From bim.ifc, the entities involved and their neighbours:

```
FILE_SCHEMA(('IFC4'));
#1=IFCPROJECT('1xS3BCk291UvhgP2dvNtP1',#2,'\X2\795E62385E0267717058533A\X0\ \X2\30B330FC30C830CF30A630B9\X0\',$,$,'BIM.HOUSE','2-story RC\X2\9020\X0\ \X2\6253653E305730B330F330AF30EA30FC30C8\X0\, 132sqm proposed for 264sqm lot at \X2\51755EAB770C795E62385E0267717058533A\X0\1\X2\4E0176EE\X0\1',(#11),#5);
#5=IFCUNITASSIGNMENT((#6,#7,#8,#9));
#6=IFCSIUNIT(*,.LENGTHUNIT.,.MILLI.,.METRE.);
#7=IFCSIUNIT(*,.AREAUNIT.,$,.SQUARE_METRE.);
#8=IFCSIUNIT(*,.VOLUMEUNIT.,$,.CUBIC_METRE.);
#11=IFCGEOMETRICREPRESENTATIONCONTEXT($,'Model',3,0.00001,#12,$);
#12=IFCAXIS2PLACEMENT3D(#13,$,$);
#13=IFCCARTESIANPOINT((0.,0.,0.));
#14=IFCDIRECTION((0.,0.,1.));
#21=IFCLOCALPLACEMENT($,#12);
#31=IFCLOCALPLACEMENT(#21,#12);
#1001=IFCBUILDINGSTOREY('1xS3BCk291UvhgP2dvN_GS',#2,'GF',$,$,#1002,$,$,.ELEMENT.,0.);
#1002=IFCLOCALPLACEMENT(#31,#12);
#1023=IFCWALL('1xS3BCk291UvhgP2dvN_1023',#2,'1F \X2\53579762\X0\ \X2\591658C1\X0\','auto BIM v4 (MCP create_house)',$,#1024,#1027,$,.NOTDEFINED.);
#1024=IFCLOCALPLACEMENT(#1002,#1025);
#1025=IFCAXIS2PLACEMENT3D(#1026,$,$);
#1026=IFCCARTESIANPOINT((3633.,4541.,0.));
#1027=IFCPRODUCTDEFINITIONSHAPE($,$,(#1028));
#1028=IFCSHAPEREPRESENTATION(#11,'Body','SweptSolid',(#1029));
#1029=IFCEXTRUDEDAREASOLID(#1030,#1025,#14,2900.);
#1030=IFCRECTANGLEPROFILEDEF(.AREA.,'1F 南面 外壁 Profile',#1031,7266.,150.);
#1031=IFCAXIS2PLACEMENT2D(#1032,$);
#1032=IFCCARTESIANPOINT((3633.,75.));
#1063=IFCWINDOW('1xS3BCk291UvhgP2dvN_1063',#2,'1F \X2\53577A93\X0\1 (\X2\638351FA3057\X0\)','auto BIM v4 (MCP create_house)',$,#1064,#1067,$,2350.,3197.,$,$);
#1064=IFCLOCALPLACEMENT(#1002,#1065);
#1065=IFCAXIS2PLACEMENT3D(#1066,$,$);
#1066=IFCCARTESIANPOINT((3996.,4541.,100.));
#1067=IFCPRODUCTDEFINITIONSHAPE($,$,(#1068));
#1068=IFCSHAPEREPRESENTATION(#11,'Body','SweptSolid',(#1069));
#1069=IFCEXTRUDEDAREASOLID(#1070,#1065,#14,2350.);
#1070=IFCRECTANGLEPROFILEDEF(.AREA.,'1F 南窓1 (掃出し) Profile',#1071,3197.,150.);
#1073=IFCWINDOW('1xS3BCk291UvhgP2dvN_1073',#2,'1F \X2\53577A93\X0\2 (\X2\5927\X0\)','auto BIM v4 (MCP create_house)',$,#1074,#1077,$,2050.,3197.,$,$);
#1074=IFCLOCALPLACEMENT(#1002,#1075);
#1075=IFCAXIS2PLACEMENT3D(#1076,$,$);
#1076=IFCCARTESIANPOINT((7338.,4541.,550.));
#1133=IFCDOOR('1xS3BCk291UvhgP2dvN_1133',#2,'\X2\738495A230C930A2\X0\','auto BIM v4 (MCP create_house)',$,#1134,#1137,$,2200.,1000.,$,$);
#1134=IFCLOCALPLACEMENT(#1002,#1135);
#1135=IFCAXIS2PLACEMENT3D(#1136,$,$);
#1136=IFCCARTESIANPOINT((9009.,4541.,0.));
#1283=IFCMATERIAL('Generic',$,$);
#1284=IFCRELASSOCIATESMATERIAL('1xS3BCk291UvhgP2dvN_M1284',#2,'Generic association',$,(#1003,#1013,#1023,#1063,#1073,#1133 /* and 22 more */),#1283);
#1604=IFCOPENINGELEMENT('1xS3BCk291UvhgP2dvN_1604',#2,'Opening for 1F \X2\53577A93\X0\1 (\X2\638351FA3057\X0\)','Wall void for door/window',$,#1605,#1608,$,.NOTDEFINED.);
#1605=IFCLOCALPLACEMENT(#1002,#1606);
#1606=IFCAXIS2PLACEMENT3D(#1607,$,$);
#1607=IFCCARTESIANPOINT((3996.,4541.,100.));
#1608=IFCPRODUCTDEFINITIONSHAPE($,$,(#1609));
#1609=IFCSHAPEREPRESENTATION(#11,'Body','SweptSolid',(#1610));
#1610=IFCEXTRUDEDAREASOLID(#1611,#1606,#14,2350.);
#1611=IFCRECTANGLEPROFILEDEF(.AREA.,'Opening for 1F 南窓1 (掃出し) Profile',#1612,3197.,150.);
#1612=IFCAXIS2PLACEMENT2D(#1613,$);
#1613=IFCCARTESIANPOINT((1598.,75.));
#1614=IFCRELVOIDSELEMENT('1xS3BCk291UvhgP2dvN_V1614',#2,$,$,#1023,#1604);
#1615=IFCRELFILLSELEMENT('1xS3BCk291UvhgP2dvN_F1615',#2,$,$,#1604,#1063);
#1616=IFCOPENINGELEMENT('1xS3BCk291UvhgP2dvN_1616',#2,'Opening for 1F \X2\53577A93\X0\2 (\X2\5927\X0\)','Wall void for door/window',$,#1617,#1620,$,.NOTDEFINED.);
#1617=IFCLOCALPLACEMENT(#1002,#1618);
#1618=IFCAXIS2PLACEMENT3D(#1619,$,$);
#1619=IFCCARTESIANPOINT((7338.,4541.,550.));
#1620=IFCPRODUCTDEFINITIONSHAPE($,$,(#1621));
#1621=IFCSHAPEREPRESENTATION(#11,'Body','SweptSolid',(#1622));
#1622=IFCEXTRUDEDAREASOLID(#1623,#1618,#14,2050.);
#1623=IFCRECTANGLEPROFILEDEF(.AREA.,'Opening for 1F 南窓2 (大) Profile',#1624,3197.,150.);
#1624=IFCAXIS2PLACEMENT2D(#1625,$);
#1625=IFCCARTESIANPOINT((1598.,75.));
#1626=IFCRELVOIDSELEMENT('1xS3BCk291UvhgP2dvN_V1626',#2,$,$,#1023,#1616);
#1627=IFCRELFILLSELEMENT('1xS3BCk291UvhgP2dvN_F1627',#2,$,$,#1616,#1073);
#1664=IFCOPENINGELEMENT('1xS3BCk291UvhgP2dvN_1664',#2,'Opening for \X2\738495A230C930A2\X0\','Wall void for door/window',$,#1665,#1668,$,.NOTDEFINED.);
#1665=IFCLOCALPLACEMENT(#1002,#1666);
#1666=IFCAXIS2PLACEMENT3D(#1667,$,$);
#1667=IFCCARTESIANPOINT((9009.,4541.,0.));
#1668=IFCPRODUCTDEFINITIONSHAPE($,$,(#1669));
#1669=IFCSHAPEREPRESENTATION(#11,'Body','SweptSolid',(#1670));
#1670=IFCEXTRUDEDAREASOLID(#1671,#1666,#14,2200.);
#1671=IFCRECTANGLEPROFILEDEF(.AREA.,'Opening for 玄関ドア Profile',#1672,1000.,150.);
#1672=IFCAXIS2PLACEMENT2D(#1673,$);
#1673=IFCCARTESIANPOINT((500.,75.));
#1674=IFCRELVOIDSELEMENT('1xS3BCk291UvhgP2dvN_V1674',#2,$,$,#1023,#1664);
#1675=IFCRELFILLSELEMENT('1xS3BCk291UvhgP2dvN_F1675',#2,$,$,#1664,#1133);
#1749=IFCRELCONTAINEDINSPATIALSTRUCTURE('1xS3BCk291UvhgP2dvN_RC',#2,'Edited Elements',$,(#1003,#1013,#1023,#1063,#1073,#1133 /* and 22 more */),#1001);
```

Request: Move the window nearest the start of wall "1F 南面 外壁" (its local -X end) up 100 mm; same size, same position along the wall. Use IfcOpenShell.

```python
import numpy as np
import ifcopenshell
import ifcopenshell.api.geometry
import ifcopenshell.util.placement
import ifcopenshell.util.unit

model = ifcopenshell.open("bim.ifc")
unit_scale = ifcopenshell.util.unit.calculate_unit_scale(model)

window = model.by_guid("1xS3BCk291UvhgP2dvN_1063")
opening = window.FillsVoids[0].RelatingOpeningElement
dz = 0.1 / unit_scale

shift = np.array([0.0, 0.0, dz])
# The window is not placed relative to its opening, so move both.
for product in (opening, window):
    matrix = ifcopenshell.util.placement.get_local_placement(product.ObjectPlacement)
    matrix[:3, 3] += shift
    ifcopenshell.api.geometry.edit_object_placement(model, product=product, matrix=matrix, is_si=False)

print(f"moved by {dz * unit_scale:+.3f} m")

model.write("bim-out.ifc")
```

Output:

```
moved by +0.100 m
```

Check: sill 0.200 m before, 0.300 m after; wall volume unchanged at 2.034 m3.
